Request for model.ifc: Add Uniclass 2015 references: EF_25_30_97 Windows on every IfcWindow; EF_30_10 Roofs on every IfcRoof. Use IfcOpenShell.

First a look at what the model holds.

```python
import ifcopenshell

model = ifcopenshell.open("model.ifc")
print(model.schema)
print("classifications:", [c.Name for c in model.by_type("IfcClassification")])
for ifc_class in ("IfcDoor", "IfcRoof", "IfcStair", "IfcWall", "IfcWindow"):
    print(ifc_class, len(model.by_type(ifc_class)))
```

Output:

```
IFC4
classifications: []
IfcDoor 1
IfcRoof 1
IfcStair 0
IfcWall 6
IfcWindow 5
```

```python
import ifcopenshell
import ifcopenshell.api.classification

model = ifcopenshell.open("model.ifc")

system = ifcopenshell.api.classification.add_classification(model, classification="Uniclass 2015")

codes = {
    "IfcWindow": ("EF_25_30_97", "Windows"),
    "IfcRoof": ("EF_30_10", "Roofs"),
}
for ifc_class, (code, name) in codes.items():
    products = model.by_type(ifc_class)
    ifcopenshell.api.classification.add_reference(
        model, products=products, classification=system, identification=code, name=name
    )
    print(code, len(products))

model.write("model_updated.ifc")
```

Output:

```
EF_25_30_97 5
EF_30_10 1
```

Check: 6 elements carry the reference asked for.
